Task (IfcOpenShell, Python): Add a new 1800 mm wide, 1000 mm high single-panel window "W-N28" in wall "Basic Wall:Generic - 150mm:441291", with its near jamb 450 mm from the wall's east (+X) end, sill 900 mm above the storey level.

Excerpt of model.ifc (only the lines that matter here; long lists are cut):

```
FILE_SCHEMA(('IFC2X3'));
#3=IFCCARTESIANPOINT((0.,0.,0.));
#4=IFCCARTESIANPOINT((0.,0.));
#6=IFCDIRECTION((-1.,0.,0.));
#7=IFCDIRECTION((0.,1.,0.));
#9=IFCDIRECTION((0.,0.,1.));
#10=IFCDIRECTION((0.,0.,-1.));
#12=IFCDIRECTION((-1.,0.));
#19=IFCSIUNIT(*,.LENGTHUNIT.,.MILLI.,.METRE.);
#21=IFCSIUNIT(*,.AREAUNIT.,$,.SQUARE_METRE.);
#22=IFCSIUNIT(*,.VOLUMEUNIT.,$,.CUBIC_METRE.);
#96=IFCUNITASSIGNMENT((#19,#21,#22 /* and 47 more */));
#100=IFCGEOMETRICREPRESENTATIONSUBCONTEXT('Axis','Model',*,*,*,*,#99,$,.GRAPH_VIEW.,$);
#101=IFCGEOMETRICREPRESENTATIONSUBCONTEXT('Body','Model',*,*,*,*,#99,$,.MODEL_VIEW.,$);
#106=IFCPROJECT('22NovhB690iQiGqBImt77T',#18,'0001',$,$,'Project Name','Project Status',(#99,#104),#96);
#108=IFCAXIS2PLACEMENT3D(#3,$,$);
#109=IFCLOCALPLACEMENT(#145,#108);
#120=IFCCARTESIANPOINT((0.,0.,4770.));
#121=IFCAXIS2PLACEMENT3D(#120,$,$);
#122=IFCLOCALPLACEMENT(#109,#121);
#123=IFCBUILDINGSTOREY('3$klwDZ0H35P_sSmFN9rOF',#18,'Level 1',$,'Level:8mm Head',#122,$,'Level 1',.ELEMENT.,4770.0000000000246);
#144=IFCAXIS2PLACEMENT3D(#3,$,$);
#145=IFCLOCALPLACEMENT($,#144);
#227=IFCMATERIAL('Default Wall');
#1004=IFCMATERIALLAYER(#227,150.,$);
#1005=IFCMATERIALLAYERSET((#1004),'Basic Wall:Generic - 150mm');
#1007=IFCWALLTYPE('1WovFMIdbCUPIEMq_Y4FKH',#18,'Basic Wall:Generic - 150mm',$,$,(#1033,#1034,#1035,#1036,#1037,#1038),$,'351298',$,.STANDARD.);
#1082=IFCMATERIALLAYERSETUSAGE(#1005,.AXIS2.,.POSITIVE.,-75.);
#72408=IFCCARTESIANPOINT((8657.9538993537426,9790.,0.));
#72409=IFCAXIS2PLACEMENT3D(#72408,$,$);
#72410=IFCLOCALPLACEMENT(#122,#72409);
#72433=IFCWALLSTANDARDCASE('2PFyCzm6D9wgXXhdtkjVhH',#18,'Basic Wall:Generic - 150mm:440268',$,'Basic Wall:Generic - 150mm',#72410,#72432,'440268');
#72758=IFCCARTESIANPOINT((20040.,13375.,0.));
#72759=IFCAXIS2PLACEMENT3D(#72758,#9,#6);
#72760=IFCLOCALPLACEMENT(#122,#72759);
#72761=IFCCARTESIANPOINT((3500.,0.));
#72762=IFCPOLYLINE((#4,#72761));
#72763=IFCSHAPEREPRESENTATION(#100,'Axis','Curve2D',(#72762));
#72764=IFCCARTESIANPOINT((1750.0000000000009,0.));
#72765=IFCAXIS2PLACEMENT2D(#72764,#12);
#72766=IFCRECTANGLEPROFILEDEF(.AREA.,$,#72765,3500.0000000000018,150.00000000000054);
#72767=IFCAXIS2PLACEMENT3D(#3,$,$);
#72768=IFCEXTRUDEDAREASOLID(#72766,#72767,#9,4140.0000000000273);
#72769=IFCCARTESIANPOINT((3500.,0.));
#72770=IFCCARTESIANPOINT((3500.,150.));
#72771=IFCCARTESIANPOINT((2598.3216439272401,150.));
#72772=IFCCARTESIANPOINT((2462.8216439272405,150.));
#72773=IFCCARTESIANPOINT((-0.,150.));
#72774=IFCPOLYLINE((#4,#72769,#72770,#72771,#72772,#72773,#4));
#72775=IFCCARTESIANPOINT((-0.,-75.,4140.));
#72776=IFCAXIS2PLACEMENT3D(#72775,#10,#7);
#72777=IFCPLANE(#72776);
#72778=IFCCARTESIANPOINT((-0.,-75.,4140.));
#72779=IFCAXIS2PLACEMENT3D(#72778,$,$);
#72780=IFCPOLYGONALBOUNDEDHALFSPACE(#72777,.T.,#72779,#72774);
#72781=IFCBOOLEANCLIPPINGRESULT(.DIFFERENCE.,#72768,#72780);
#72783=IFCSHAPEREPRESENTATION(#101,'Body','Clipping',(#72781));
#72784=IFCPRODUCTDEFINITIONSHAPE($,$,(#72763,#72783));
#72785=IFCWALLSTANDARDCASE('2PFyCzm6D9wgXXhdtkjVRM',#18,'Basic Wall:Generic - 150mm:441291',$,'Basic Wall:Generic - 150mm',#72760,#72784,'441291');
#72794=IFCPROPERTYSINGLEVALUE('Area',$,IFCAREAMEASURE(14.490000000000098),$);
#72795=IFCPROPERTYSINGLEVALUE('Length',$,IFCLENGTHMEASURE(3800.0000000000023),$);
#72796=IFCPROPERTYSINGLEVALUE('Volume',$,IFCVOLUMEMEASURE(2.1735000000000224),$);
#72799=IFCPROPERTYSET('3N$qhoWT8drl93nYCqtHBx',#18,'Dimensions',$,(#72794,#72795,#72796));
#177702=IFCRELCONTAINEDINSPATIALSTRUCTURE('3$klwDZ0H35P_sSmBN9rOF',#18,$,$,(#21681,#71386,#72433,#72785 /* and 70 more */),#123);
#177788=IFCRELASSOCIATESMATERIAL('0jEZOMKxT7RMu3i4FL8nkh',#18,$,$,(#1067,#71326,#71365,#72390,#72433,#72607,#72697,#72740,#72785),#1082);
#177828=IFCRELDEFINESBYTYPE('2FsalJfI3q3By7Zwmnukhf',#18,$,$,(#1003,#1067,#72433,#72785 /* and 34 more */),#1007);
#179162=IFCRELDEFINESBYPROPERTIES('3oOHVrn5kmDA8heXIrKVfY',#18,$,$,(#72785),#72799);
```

```python
import numpy as np
import ifcopenshell
import ifcopenshell.api.feature
import ifcopenshell.api.geometry
import ifcopenshell.api.pset
import ifcopenshell.api.root
import ifcopenshell.api.spatial
import ifcopenshell.api.type
import ifcopenshell.geom
import ifcopenshell.util.element
import ifcopenshell.util.placement
import ifcopenshell.util.representation
import ifcopenshell.util.shape
import ifcopenshell.util.unit

model = ifcopenshell.open("model.ifc")
unit_scale = ifcopenshell.util.unit.calculate_unit_scale(model)
area_scale = ifcopenshell.util.unit.calculate_unit_scale(model, "AREAUNIT")
volume_scale = ifcopenshell.util.unit.calculate_unit_scale(model, "VOLUMEUNIT")
settings = ifcopenshell.geom.settings()


def volume(element):
    """Net volume in cubic metres, openings subtracted."""
    shape = ifcopenshell.geom.create_shape(settings, element)
    return ifcopenshell.util.shape.get_volume(shape.geometry)


wall = model.by_guid("2PFyCzm6D9wgXXhdtkjVRM")
storey = ifcopenshell.util.element.get_container(wall, ifc_class="IfcBuildingStorey")
context = ifcopenshell.util.representation.get_context(model, "Model", "Body", "MODEL_VIEW")
before = volume(wall)

width, height, from_end, sill = 1.8, 1, 0.45, 0.9  # metres

# The wall runs along its own X axis, and the end named is its -X end.
wall_shape = ifcopenshell.geom.create_shape(settings, wall)
x, y, z = ifcopenshell.util.shape.get_vertices(wall_shape.geometry).T
start = x.min() + from_end
face, thickness = float(y.min()), float(y.max() - y.min())
wall_matrix = ifcopenshell.util.placement.get_local_placement(wall.ObjectPlacement)
level = ifcopenshell.util.placement.get_local_placement(storey.ObjectPlacement)[2, 3]


def in_wall(x, y):
    """Placement at x, y metres in the wall's axes, at sill height."""
    matrix = wall_matrix.copy()
    matrix[:, 3] = wall_matrix @ np.array([x / unit_scale, y / unit_scale, 0.0, 1.0])
    matrix[2, 3] = level + sill / unit_scale
    return matrix


# Opening: a box that overshoots both wall faces by 50 mm.
opening = ifcopenshell.api.root.create_entity(model, ifc_class="IfcOpeningElement")
box = ifcopenshell.api.geometry.add_wall_representation(
    model, context=context, length=width, height=height, thickness=thickness + 0.1
)
ifcopenshell.api.geometry.assign_representation(model, product=opening, representation=box)
ifcopenshell.api.geometry.edit_object_placement(model, product=opening, matrix=in_wall(start, face - 0.05), is_si=False)
ifcopenshell.api.feature.add_feature(model, feature=opening, element=wall)

window = ifcopenshell.api.root.create_entity(model, ifc_class="IfcWindow", name="W-N28")
window.OverallWidth, window.OverallHeight = width / unit_scale, height / unit_scale
body = ifcopenshell.api.geometry.add_window_representation(
    model,
    context=context,
    overall_width=window.OverallWidth,
    overall_height=window.OverallHeight,
    partition_type="SINGLE_PANEL",
)
ifcopenshell.api.geometry.assign_representation(model, product=window, representation=body)
ifcopenshell.api.spatial.assign_container(model, products=[window], relating_structure=storey)
fills = ifcopenshell.api.feature.add_filling(model, opening=opening, element=window)
fills.OwnerHistory = window.OwnerHistory  # required in IFC2X3

# IFC2X3 keeps the operation on the window style.
style = ifcopenshell.api.root.create_entity(model, ifc_class="IfcWindowStyle", name="W-N28")
style.OperationType, style.ConstructionType = "SINGLE_PANEL", "NOTDEFINED"
style.ParameterTakesPrecedence = style.Sizeable = False
ifcopenshell.api.type.assign_type(model, related_objects=[window], relating_type=style)

# Centre the window in the wall's thickness.
ifcopenshell.api.geometry.edit_object_placement(model, product=window, matrix=in_wall(start, face), is_si=False)
window_shape = ifcopenshell.geom.create_shape(settings, window)
depth = ifcopenshell.util.shape.get_vertices(window_shape.geometry)[:, 1]
offset = face + thickness / 2 - (depth.min() + depth.max()) / 2
ifcopenshell.api.geometry.edit_object_placement(model, product=window, matrix=in_wall(start, offset), is_si=False)

after = volume(wall)

# Update the wall's stored quantities.
pset = model.by_id(ifcopenshell.util.element.get_pset(wall, "Dimensions", should_inherit=False)["id"])
ifcopenshell.api.pset.edit_pset(model, pset=pset, properties={
    "Area": model.create_entity("IfcAreaMeasure", after / thickness / area_scale),
    "Volume": model.create_entity("IfcVolumeMeasure", after / volume_scale),
})

print(f"wall volume {before:.3f} -> {after:.3f} m3")

model.write("model_edited.ifc")
```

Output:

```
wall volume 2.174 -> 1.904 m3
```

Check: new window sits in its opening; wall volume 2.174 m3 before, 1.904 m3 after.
